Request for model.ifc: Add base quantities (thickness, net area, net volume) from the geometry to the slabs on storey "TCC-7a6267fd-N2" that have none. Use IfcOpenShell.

First a look at what the model holds.

```python
import ifcopenshell
import ifcopenshell.util.element
import ifcopenshell.util.unit

model = ifcopenshell.open("model.ifc")
print(model.schema)
for unit_type in ("LENGTHUNIT", "AREAUNIT", "VOLUMEUNIT"):
    print(unit_type, ifcopenshell.util.unit.calculate_unit_scale(model, unit_type))
storey = next(s for s in model.by_type("IfcBuildingStorey") if s.Name == "TCC-7a6267fd-N2")
slabs = [e for e in ifcopenshell.util.element.get_decomposition(storey) if e.is_a("IfcSlab")]
for e in sorted(slabs, key=lambda e: e.id()):
    print(e.id(), e.is_a(), e.Name, list(ifcopenshell.util.element.get_psets(e, qtos_only=True)), sep=" | ")
```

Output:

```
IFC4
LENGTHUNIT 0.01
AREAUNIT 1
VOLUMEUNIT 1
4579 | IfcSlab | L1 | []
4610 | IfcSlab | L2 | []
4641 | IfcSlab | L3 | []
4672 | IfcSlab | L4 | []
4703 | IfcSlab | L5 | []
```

```python
import ifcopenshell
import ifcopenshell.api.pset
import ifcopenshell.geom
import ifcopenshell.util.element
import ifcopenshell.util.shape
import ifcopenshell.util.unit

model = ifcopenshell.open("model.ifc")
unit_scale = ifcopenshell.util.unit.calculate_unit_scale(model)
area_scale = ifcopenshell.util.unit.calculate_unit_scale(model, "AREAUNIT")
volume_scale = ifcopenshell.util.unit.calculate_unit_scale(model, "VOLUMEUNIT")
settings = ifcopenshell.geom.settings()

storey = next(s for s in model.by_type("IfcBuildingStorey") if s.Name == "TCC-7a6267fd-N2")
slabs = [e for e in ifcopenshell.util.element.get_decomposition(storey) if e.is_a("IfcSlab")]

for e in sorted(slabs, key=lambda e: e.id()):
    if ifcopenshell.util.element.get_psets(e, qtos_only=True, should_inherit=False):
        continue
    # Geometry comes back in metres, in the element's own axes.
    shape = ifcopenshell.geom.create_shape(settings, e)
    values = {
        "Width": ifcopenshell.util.shape.get_z(shape.geometry) / unit_scale,
        "NetArea": ifcopenshell.util.shape.get_footprint_area(shape.geometry) / area_scale,
        "NetVolume": ifcopenshell.util.shape.get_volume(shape.geometry) / volume_scale,
    }
    qto = ifcopenshell.api.pset.add_qto(model, product=e, name="Qto_SlabBaseQuantities")
    ifcopenshell.api.pset.edit_qto(model, qto=qto, properties=values)
    print(e.id(), {k: round(v, 3) for k, v in values.items()})

model.write("model_v2.ifc")
```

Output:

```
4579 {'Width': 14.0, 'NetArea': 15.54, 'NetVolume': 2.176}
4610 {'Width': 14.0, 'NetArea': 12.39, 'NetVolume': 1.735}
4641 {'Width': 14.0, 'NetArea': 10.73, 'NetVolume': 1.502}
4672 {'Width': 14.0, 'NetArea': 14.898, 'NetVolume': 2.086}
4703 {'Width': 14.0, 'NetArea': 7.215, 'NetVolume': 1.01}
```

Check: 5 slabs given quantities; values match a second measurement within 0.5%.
